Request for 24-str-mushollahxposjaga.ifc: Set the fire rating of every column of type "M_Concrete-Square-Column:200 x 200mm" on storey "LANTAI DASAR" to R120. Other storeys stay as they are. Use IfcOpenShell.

First a look at what the model holds.

```python
import ifcopenshell
import ifcopenshell.util.element

model = ifcopenshell.open("24-str-mushollahxposjaga.ifc")
print(model.schema)
storey = next(s for s in model.by_type("IfcBuildingStorey") if s.Name == "LANTAI DASAR")
columns = [e for e in ifcopenshell.util.element.get_decomposition(storey) if e.is_a("IfcColumn")]
seen = {}
for e in columns:
    element_type = ifcopenshell.util.element.get_type(e)
    key = (element_type.Name if element_type != e and element_type else None, ifcopenshell.util.element.get_pset(e, "Pset_ColumnCommon", "FireRating"))
    seen[key] = seen.get(key, 0) + 1
for (name, value), count in sorted(seen.items(), key=str):
    print(count, "x", name, "|", value)
```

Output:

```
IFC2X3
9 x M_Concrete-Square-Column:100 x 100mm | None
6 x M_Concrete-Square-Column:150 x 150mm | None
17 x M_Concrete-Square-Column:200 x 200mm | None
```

```python
import ifcopenshell
import ifcopenshell.api.pset
import ifcopenshell.util.element

model = ifcopenshell.open("24-str-mushollahxposjaga.ifc")

storey = next(s for s in model.by_type("IfcBuildingStorey") if s.Name == "LANTAI DASAR")
columns = [e for e in ifcopenshell.util.element.get_decomposition(storey) if e.is_a("IfcColumn")]

count = 0
for e in columns:
    element_type = ifcopenshell.util.element.get_type(e)
    if element_type in (None, e) or element_type.Name != "M_Concrete-Square-Column:200 x 200mm":
        continue
    # add_pset returns the element's existing set when there is one.
    pset = ifcopenshell.api.pset.add_pset(model, product=e, name="Pset_ColumnCommon")
    ifcopenshell.api.pset.edit_pset(model, pset=pset, properties={"FireRating": "R120"})
    count += 1

print(count, "columns updated")

model.write("24-str-mushollahxposjaga_edited.ifc")
```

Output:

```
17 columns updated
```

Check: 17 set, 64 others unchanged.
